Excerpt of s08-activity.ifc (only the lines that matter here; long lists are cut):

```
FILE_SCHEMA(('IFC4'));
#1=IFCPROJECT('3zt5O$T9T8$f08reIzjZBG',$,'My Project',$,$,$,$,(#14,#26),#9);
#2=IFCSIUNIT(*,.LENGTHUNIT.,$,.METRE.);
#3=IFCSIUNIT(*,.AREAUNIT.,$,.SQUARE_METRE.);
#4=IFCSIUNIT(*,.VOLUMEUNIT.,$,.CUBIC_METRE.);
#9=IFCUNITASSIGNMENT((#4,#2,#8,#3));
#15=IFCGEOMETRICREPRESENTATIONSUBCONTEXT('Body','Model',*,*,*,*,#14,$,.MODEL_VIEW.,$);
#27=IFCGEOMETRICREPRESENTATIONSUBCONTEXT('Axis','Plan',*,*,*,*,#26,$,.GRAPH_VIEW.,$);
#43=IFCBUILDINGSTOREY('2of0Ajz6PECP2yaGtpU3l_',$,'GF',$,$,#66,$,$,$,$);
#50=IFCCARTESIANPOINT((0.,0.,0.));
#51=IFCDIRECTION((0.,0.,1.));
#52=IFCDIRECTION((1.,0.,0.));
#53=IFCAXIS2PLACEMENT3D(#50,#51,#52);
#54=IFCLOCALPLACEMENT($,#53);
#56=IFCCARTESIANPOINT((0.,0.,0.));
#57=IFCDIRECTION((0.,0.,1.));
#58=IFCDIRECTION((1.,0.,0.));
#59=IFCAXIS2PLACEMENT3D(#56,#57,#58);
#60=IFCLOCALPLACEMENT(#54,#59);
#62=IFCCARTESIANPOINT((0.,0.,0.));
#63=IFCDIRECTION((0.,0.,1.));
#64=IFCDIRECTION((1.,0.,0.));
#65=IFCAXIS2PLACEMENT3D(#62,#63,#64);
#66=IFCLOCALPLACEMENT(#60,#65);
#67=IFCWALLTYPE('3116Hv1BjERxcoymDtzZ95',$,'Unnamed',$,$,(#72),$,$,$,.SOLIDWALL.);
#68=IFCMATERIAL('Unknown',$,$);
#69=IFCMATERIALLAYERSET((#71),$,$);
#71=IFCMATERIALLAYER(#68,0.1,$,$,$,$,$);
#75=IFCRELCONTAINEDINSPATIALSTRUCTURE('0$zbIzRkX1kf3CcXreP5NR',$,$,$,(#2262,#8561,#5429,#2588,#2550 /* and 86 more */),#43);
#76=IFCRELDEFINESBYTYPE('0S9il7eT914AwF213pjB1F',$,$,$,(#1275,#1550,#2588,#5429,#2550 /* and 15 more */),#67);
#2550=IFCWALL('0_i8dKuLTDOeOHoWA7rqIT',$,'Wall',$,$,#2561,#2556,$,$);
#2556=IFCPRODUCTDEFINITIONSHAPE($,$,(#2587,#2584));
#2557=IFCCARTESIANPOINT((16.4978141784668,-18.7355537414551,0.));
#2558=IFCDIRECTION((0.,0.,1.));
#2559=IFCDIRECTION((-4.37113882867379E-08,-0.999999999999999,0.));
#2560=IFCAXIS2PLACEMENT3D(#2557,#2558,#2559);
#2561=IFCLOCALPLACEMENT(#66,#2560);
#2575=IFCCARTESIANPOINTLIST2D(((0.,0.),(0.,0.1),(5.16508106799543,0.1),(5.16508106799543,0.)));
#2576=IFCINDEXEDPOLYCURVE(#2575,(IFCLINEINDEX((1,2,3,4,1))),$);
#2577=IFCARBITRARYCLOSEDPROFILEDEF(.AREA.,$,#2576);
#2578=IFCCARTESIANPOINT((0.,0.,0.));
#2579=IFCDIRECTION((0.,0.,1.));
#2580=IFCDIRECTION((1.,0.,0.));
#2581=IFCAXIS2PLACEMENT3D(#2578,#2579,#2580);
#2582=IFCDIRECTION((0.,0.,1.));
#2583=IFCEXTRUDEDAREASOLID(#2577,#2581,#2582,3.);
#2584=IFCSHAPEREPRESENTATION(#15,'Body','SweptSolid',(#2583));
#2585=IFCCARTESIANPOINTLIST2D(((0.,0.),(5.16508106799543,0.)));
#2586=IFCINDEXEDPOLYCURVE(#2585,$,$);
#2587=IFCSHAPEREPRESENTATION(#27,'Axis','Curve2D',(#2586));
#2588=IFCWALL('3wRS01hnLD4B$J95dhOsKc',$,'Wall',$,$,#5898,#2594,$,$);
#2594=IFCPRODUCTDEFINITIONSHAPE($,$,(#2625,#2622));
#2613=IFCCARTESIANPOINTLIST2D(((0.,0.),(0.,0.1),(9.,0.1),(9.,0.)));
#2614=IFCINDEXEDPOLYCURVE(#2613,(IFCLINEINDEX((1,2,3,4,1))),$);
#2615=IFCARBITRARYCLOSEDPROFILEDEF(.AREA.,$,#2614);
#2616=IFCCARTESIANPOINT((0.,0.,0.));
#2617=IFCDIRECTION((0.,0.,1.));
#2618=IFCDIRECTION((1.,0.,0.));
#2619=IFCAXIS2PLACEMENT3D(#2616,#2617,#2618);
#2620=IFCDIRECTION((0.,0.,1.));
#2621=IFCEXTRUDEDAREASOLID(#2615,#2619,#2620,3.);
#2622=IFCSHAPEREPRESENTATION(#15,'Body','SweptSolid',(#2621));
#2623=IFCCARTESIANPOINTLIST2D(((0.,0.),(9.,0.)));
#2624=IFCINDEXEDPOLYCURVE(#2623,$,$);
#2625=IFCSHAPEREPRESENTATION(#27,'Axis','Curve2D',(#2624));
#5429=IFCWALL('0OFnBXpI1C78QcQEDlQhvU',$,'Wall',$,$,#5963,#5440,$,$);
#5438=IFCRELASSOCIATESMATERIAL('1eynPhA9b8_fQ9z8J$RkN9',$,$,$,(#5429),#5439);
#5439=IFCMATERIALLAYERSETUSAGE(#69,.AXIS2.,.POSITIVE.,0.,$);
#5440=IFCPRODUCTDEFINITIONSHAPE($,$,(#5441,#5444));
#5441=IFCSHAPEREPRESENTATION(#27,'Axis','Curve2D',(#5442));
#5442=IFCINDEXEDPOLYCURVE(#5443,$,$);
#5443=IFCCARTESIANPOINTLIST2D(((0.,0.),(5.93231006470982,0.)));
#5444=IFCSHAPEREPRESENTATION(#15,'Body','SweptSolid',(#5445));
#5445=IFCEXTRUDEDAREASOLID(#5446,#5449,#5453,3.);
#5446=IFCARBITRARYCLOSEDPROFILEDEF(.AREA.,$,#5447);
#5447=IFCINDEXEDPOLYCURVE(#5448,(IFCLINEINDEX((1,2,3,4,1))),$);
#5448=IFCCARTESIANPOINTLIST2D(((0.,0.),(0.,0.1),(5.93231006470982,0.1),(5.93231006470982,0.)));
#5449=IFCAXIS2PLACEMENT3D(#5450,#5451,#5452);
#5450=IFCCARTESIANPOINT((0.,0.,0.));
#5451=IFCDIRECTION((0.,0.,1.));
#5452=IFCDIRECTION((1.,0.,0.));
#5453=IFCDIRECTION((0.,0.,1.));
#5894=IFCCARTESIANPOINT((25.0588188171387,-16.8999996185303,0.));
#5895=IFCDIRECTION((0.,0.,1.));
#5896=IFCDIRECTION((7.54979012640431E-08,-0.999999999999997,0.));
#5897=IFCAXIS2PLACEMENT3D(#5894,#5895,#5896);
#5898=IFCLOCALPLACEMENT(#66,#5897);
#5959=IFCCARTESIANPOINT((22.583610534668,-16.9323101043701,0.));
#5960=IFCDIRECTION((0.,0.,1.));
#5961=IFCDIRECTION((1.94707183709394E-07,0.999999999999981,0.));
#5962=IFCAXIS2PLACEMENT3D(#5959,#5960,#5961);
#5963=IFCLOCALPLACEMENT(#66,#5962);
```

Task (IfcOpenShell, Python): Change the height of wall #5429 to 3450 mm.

```python
import ifcopenshell
import ifcopenshell.geom
import ifcopenshell.util.representation
import ifcopenshell.util.shape
import ifcopenshell.util.unit

model = ifcopenshell.open("s08-activity.ifc")
unit_scale = ifcopenshell.util.unit.calculate_unit_scale(model)
settings = ifcopenshell.geom.settings()


def volume(element):
    """Net volume in cubic metres, openings subtracted."""
    shape = ifcopenshell.geom.create_shape(settings, element)
    return ifcopenshell.util.shape.get_volume(shape.geometry)


wall = model.by_guid("0OFnBXpI1C78QcQEDlQhvU")
before = volume(wall)

body = ifcopenshell.util.representation.get_representation(wall, "Model", "Body")
solid = body.Items[0]
old_height = solid.Depth
solid.Depth = 3.45 / unit_scale
after = volume(wall)

print(f"height {old_height:g} -> {solid.Depth:g}, volume {before:.3f} -> {after:.3f} m3")

model.write("s08-activity_rev.ifc")
```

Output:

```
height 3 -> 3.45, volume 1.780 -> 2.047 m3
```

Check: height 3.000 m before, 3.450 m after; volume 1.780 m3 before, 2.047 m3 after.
